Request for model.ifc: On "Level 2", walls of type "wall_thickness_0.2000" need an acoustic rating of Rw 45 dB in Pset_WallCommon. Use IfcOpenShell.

First a look at what the model holds.

```python
import ifcopenshell
import ifcopenshell.util.element

model = ifcopenshell.open("model.ifc")
print(model.schema)
storey = next(s for s in model.by_type("IfcBuildingStorey") if s.Name == "Level 2")
walls = [e for e in ifcopenshell.util.element.get_decomposition(storey) if e.is_a("IfcWall")]
seen = {}
for e in walls:
    element_type = ifcopenshell.util.element.get_type(e)
    key = (element_type.Name if element_type != e and element_type else None, ifcopenshell.util.element.get_pset(e, "Pset_WallCommon", "AcousticRating"))
    seen[key] = seen.get(key, 0) + 1
for (name, value), count in sorted(seen.items(), key=str):
    print(count, "x", name, "|", value)
```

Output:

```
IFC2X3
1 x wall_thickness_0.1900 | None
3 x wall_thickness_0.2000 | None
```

```python
import ifcopenshell
import ifcopenshell.api.pset
import ifcopenshell.util.element

model = ifcopenshell.open("model.ifc")

storey = next(s for s in model.by_type("IfcBuildingStorey") if s.Name == "Level 2")
walls = [e for e in ifcopenshell.util.element.get_decomposition(storey) if e.is_a("IfcWall")]

count = 0
for e in walls:
    element_type = ifcopenshell.util.element.get_type(e)
    if element_type in (None, e) or element_type.Name != "wall_thickness_0.2000":
        continue
    # add_pset returns the element's existing set when there is one.
    pset = ifcopenshell.api.pset.add_pset(model, product=e, name="Pset_WallCommon")
    ifcopenshell.api.pset.edit_pset(model, pset=pset, properties={"AcousticRating": "Rw 45 dB"})
    count += 1

print(count, "walls updated")

model.write("model_updated.ifc")
```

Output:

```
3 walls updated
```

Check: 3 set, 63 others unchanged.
